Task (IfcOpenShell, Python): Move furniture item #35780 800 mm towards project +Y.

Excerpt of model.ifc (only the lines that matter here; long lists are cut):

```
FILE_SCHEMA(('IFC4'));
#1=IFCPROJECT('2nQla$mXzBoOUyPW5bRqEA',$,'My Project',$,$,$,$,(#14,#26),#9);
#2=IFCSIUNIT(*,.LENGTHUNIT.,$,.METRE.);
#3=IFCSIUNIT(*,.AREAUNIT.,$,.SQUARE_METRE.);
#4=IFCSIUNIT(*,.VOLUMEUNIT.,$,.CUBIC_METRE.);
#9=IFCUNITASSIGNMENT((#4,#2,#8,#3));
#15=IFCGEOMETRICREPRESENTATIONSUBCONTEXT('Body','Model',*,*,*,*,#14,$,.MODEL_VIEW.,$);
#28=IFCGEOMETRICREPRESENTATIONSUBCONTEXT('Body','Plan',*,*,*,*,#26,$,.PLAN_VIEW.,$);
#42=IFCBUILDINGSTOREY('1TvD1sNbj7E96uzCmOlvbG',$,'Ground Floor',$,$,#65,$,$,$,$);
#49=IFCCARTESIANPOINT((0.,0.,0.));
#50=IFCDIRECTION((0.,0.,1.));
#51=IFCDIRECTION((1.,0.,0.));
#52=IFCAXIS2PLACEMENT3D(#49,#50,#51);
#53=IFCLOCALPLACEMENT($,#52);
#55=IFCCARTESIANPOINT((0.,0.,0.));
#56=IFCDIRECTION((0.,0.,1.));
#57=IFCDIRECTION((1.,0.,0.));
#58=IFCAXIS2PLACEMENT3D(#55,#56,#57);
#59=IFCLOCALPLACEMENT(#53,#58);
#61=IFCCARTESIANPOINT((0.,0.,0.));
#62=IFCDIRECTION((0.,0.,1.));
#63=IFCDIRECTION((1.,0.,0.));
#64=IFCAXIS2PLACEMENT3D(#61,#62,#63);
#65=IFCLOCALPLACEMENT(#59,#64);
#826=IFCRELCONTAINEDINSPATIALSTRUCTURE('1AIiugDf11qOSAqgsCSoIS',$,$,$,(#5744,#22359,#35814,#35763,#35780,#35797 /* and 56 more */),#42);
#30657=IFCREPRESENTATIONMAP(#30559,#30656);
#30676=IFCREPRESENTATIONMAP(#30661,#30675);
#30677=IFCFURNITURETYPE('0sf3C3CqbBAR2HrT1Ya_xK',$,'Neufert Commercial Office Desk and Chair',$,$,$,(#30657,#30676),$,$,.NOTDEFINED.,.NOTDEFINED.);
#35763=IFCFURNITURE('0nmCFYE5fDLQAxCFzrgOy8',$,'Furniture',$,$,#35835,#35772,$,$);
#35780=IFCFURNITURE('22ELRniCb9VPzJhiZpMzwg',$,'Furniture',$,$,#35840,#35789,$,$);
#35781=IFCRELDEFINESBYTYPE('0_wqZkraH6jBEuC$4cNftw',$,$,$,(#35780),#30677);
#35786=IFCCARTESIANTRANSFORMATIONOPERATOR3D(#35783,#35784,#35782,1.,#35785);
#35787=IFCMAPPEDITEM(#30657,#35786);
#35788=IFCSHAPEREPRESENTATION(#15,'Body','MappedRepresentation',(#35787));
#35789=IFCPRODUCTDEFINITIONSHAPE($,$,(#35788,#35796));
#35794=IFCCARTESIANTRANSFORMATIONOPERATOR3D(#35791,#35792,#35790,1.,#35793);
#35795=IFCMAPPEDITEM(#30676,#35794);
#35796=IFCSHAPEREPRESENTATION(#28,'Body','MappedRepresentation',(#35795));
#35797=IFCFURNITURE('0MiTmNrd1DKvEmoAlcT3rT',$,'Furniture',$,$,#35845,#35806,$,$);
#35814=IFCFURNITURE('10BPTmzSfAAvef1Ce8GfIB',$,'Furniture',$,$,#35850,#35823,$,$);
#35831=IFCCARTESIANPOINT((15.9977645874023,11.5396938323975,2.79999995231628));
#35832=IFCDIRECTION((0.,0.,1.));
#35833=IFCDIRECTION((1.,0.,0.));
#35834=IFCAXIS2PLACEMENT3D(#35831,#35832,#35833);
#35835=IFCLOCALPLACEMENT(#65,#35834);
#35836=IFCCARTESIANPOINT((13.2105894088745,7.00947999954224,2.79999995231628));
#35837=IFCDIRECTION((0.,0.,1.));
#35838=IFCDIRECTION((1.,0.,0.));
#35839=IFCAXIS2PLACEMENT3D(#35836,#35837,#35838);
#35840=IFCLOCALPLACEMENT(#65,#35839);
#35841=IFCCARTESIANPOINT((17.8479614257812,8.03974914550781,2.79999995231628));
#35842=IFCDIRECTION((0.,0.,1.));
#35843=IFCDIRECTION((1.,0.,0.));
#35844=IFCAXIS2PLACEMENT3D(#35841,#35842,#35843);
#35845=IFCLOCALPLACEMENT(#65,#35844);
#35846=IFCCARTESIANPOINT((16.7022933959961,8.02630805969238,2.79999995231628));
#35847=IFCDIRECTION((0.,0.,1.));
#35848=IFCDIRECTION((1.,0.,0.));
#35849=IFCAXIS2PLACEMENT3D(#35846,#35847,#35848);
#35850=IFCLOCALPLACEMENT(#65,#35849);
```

```python
import ifcopenshell
import ifcopenshell.api.geometry
import ifcopenshell.util.placement
import ifcopenshell.util.unit

model = ifcopenshell.open("model.ifc")
unit_scale = ifcopenshell.util.unit.calculate_unit_scale(model)

item = model.by_guid("22ELRniCb9VPzJhiZpMzwg")
matrix = ifcopenshell.util.placement.get_local_placement(item.ObjectPlacement)
matrix[1, 3] += 0.8 / unit_scale
ifcopenshell.api.geometry.edit_object_placement(model, product=item, matrix=matrix, is_si=False)

print(ifcopenshell.util.placement.get_local_placement(item.ObjectPlacement).round(3) + 0.0)

model.write("model-out.ifc")
```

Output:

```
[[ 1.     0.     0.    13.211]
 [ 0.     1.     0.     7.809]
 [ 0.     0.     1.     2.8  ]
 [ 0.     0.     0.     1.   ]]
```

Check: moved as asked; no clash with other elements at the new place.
